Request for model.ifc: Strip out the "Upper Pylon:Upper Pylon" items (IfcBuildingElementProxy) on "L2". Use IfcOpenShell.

First a look at what the model holds.

```python
import ifcopenshell
import ifcopenshell.util.element

model = ifcopenshell.open("model.ifc")
print(model.schema)
storey = next(s for s in model.by_type("IfcBuildingStorey") if s.Name == "L2")
proxies = [e for e in ifcopenshell.util.element.get_decomposition(storey) if e.is_a("IfcBuildingElementProxy")]
seen = {}
for e in proxies:
    element_type = ifcopenshell.util.element.get_type(e)
    name = element_type.Name if element_type not in (None, e) else None
    seen[name] = seen.get(name, 0) + 1
for name, count in sorted(seen.items(), key=str):
    print(count, "x", name)
```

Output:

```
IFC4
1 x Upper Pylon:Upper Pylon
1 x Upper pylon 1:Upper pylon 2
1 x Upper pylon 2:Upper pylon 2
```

```python
import ifcopenshell
import ifcopenshell.api.root
import ifcopenshell.util.element

model = ifcopenshell.open("model.ifc")

storey = next(s for s in model.by_type("IfcBuildingStorey") if s.Name == "L2")
proxies = [e for e in ifcopenshell.util.element.get_decomposition(storey) if e.is_a("IfcBuildingElementProxy")]
targets = [e for e in proxies if (t := ifcopenshell.util.element.get_type(e)) not in (None, e) and t.Name == "Upper Pylon:Upper Pylon"]

for e in targets:
    ifcopenshell.api.root.remove_product(model, product=e)
print(len(targets), "removed")

model.write("model_edited.ifc")
```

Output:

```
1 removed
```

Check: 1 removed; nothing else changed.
